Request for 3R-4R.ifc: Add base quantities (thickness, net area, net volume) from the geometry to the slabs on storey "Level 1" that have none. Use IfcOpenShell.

First a look at what the model holds.

```python
import ifcopenshell
import ifcopenshell.util.element
import ifcopenshell.util.unit

model = ifcopenshell.open("3R-4R.ifc")
print(model.schema)
for unit_type in ("LENGTHUNIT", "AREAUNIT", "VOLUMEUNIT"):
    print(unit_type, ifcopenshell.util.unit.calculate_unit_scale(model, unit_type))
storey = next(s for s in model.by_type("IfcBuildingStorey") if s.Name == "Level 1")
slabs = [e for e in ifcopenshell.util.element.get_decomposition(storey) if e.is_a("IfcSlab")]
for e in sorted(slabs, key=lambda e: e.id()):
    print(e.id(), e.is_a(), e.Name, list(ifcopenshell.util.element.get_psets(e, qtos_only=True)), sep=" | ")
```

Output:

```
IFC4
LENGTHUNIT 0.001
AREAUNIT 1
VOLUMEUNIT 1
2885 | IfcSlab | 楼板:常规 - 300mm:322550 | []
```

```python
import ifcopenshell
import ifcopenshell.api.pset
import ifcopenshell.geom
import ifcopenshell.util.element
import ifcopenshell.util.shape
import ifcopenshell.util.unit

model = ifcopenshell.open("3R-4R.ifc")
unit_scale = ifcopenshell.util.unit.calculate_unit_scale(model)
area_scale = ifcopenshell.util.unit.calculate_unit_scale(model, "AREAUNIT")
volume_scale = ifcopenshell.util.unit.calculate_unit_scale(model, "VOLUMEUNIT")
settings = ifcopenshell.geom.settings()

storey = next(s for s in model.by_type("IfcBuildingStorey") if s.Name == "Level 1")
slabs = [e for e in ifcopenshell.util.element.get_decomposition(storey) if e.is_a("IfcSlab")]

for e in sorted(slabs, key=lambda e: e.id()):
    if ifcopenshell.util.element.get_psets(e, qtos_only=True, should_inherit=False):
        continue
    # Geometry comes back in metres, in the element's own axes.
    shape = ifcopenshell.geom.create_shape(settings, e)
    values = {
        "Width": ifcopenshell.util.shape.get_z(shape.geometry) / unit_scale,
        "NetArea": ifcopenshell.util.shape.get_footprint_area(shape.geometry) / area_scale,
        "NetVolume": ifcopenshell.util.shape.get_volume(shape.geometry) / volume_scale,
    }
    qto = ifcopenshell.api.pset.add_qto(model, product=e, name="Qto_SlabBaseQuantities")
    ifcopenshell.api.pset.edit_qto(model, qto=qto, properties=values)
    print(e.id(), {k: round(v, 3) for k, v in values.items()})

model.write("3R-4R_edited.ifc")
```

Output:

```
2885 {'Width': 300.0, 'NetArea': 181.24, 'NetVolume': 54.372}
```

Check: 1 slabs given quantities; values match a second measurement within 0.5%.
